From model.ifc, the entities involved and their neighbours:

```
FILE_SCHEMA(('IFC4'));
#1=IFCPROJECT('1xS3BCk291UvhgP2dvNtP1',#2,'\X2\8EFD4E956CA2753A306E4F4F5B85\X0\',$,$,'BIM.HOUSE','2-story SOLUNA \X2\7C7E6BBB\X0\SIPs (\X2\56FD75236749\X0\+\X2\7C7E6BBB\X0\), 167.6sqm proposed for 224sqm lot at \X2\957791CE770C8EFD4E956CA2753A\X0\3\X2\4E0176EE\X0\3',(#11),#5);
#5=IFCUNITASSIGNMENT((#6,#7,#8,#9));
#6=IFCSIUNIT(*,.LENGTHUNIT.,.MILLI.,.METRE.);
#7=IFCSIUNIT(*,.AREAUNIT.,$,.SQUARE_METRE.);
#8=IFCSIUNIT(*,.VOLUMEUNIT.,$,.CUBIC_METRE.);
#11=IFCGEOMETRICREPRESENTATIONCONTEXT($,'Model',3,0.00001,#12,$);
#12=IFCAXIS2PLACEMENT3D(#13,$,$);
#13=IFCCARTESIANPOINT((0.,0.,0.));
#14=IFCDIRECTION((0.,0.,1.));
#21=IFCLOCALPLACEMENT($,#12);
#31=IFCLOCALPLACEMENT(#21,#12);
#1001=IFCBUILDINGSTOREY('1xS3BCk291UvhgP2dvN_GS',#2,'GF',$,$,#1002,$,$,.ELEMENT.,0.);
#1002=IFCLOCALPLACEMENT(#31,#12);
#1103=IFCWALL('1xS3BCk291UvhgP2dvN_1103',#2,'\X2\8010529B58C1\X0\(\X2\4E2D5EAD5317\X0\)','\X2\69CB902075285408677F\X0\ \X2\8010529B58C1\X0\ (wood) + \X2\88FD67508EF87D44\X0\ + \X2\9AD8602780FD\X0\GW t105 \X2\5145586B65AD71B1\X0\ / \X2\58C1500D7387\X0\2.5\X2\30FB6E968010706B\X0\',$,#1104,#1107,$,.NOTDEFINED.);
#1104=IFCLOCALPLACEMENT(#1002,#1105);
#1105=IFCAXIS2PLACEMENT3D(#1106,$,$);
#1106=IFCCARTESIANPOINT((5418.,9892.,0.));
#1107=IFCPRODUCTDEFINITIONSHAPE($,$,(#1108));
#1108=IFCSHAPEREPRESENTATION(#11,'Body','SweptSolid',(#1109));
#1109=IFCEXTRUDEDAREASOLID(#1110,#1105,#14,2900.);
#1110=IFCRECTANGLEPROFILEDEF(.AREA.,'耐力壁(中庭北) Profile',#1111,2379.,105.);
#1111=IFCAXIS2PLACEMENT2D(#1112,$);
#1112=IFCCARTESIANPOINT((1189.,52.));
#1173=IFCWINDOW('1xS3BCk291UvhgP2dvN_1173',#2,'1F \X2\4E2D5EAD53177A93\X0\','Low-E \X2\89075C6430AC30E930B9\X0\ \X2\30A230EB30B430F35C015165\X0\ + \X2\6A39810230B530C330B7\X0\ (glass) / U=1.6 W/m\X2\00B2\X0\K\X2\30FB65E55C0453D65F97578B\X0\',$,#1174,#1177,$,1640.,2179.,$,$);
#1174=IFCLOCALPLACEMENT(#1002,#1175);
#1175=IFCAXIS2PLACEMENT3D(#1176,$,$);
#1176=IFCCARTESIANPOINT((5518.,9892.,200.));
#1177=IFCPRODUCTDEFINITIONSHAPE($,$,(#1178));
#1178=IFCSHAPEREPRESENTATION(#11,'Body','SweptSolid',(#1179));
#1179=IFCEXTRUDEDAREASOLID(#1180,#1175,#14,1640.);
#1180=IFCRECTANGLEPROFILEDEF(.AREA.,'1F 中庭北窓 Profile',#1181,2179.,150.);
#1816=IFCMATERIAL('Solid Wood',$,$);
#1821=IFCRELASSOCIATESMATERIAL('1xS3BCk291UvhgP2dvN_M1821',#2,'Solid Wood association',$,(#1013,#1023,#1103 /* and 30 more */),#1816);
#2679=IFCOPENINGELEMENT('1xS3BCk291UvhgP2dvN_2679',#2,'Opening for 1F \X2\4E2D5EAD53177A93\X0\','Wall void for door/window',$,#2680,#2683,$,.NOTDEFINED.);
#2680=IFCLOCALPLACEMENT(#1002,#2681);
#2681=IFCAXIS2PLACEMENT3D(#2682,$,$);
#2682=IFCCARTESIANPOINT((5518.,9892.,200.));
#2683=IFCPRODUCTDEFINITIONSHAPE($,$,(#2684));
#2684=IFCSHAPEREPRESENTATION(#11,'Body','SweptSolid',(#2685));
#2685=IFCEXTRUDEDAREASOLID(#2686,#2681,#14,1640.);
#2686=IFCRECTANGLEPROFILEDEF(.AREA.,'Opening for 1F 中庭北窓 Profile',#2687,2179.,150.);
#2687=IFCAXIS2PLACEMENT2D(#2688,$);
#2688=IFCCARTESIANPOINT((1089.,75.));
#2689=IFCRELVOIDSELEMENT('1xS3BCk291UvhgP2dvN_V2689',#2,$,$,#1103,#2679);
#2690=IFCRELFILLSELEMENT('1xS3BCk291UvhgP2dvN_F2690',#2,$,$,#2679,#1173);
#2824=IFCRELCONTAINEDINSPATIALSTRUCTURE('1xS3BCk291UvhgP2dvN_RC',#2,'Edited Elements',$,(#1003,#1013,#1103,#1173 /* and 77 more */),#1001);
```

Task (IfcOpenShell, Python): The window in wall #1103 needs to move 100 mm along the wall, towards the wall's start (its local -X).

```python
import ifcopenshell
import ifcopenshell.api.geometry
import ifcopenshell.util.placement
import ifcopenshell.util.unit

model = ifcopenshell.open("model.ifc")
unit_scale = ifcopenshell.util.unit.calculate_unit_scale(model)

window = model.by_guid("1xS3BCk291UvhgP2dvN_1173")
opening = window.FillsVoids[0].RelatingOpeningElement
wall = opening.VoidsElements[0].RelatingBuildingElement

wall_matrix = ifcopenshell.util.placement.get_local_placement(wall.ObjectPlacement)
shift = wall_matrix[:3, 0] * -0.1 / unit_scale
before = ifcopenshell.util.placement.get_local_placement(window.ObjectPlacement)[:3, 3].copy()

# The window is not placed relative to its opening, so move both.
for product in (opening, window):
    matrix = ifcopenshell.util.placement.get_local_placement(product.ObjectPlacement)
    matrix[:3, 3] += shift
    ifcopenshell.api.geometry.edit_object_placement(model, product=product, matrix=matrix, is_si=False)

after = ifcopenshell.util.placement.get_local_placement(window.ObjectPlacement)[:3, 3]
print("window moved by", (after - before).round(3) + 0.0)

model.write("model-out.ifc")
```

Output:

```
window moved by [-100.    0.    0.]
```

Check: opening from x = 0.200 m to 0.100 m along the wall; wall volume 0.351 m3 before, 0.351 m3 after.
